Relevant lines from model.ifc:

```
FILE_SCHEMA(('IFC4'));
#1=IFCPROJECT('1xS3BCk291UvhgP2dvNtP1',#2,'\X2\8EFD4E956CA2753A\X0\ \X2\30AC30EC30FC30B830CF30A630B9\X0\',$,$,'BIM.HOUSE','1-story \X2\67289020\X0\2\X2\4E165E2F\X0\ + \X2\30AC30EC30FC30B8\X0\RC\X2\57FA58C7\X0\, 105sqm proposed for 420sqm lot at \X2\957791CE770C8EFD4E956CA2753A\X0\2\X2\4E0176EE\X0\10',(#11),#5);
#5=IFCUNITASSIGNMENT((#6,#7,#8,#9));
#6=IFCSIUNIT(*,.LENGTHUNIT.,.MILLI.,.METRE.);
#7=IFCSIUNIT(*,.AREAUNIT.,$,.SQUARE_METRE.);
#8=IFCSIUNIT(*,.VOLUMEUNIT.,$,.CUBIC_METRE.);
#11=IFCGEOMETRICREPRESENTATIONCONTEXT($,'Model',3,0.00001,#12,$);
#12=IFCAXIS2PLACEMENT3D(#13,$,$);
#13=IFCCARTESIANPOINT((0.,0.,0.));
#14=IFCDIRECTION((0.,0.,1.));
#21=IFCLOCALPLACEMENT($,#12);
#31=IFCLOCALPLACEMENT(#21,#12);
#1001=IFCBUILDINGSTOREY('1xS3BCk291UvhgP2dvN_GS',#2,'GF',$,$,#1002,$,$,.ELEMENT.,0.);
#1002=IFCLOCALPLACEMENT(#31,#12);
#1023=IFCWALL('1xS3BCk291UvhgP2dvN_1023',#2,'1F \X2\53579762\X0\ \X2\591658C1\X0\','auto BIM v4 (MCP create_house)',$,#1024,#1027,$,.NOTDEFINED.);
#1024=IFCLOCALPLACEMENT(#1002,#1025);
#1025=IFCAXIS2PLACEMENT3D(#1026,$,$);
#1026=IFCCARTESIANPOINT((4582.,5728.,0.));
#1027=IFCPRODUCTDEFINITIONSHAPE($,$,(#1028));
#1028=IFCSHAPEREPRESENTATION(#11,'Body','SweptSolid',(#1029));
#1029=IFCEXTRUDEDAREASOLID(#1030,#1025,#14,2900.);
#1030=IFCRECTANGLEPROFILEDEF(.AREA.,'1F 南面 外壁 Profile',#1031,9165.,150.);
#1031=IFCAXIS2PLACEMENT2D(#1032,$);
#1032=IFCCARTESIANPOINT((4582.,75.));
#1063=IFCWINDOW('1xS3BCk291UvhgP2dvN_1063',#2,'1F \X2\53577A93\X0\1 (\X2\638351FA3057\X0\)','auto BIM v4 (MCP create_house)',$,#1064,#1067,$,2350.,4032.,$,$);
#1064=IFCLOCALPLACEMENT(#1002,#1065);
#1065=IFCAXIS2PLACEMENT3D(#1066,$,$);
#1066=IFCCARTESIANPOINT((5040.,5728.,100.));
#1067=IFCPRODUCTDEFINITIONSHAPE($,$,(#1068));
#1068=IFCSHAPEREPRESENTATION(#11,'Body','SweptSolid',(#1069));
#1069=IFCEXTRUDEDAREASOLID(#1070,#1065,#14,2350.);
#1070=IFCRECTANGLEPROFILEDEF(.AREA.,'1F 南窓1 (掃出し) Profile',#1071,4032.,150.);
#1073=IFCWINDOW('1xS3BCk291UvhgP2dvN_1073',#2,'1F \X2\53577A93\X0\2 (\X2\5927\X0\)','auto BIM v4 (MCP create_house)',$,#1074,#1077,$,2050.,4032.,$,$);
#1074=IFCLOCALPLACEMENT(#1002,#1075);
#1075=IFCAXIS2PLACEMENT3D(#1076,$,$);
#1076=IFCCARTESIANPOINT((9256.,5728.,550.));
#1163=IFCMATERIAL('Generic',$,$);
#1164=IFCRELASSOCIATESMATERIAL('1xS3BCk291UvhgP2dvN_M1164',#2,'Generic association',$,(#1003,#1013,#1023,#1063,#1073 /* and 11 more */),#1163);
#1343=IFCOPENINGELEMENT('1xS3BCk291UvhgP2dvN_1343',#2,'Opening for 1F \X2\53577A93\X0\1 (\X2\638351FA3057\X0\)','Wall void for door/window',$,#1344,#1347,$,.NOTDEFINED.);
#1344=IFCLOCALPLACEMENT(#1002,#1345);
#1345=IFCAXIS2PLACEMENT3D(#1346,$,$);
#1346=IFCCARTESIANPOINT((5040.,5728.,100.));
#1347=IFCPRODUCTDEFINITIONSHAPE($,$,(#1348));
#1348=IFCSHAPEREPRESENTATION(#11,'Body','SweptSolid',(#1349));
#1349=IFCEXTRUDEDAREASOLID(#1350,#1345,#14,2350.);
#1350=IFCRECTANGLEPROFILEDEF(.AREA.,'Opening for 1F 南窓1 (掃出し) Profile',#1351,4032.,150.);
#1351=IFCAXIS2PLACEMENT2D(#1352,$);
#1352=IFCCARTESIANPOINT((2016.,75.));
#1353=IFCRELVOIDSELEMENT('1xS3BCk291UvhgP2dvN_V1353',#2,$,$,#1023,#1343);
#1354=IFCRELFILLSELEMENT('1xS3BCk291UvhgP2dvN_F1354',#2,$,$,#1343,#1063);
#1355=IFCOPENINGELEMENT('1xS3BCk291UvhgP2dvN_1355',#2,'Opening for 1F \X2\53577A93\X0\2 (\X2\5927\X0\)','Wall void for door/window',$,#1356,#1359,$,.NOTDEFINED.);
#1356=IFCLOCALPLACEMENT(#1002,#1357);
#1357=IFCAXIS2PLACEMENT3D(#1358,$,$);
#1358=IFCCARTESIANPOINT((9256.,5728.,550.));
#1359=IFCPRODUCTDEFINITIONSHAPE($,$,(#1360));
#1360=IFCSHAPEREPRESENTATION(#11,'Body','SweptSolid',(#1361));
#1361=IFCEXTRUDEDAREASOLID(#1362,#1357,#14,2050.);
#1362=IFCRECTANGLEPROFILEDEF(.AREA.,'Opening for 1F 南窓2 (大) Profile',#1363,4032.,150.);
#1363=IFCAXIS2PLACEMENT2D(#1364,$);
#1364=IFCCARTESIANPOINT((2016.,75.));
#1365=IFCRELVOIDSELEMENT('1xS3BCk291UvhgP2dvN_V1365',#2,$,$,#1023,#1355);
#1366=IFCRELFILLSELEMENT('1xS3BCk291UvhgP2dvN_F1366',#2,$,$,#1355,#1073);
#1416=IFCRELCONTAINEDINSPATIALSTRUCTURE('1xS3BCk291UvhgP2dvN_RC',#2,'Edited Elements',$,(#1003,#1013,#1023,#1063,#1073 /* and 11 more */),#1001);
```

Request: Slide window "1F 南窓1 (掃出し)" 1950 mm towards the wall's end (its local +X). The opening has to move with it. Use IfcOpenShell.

```python
import ifcopenshell
import ifcopenshell.api.geometry
import ifcopenshell.util.placement

model = ifcopenshell.open("model.ifc")

window = model.by_guid("1xS3BCk291UvhgP2dvN_1063")
opening = window.FillsVoids[0].RelatingOpeningElement
wall = opening.VoidsElements[0].RelatingBuildingElement

wall_matrix = ifcopenshell.util.placement.get_local_placement(wall.ObjectPlacement)
shift = wall_matrix[:3, 0] * 1950.0
before = ifcopenshell.util.placement.get_local_placement(window.ObjectPlacement)[:3, 3].copy()

# The window is not placed relative to its opening, so move both.
for product in (opening, window):
    matrix = ifcopenshell.util.placement.get_local_placement(product.ObjectPlacement)
    matrix[:3, 3] += shift
    ifcopenshell.api.geometry.edit_object_placement(model, product=product, matrix=matrix, is_si=False)

after = ifcopenshell.util.placement.get_local_placement(window.ObjectPlacement)[:3, 3]
print("window moved by", (after - before).round(3) + 0.0)

model.write("model_edited.ifc")
```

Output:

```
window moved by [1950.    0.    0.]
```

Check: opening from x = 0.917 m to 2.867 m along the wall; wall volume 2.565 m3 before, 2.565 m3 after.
